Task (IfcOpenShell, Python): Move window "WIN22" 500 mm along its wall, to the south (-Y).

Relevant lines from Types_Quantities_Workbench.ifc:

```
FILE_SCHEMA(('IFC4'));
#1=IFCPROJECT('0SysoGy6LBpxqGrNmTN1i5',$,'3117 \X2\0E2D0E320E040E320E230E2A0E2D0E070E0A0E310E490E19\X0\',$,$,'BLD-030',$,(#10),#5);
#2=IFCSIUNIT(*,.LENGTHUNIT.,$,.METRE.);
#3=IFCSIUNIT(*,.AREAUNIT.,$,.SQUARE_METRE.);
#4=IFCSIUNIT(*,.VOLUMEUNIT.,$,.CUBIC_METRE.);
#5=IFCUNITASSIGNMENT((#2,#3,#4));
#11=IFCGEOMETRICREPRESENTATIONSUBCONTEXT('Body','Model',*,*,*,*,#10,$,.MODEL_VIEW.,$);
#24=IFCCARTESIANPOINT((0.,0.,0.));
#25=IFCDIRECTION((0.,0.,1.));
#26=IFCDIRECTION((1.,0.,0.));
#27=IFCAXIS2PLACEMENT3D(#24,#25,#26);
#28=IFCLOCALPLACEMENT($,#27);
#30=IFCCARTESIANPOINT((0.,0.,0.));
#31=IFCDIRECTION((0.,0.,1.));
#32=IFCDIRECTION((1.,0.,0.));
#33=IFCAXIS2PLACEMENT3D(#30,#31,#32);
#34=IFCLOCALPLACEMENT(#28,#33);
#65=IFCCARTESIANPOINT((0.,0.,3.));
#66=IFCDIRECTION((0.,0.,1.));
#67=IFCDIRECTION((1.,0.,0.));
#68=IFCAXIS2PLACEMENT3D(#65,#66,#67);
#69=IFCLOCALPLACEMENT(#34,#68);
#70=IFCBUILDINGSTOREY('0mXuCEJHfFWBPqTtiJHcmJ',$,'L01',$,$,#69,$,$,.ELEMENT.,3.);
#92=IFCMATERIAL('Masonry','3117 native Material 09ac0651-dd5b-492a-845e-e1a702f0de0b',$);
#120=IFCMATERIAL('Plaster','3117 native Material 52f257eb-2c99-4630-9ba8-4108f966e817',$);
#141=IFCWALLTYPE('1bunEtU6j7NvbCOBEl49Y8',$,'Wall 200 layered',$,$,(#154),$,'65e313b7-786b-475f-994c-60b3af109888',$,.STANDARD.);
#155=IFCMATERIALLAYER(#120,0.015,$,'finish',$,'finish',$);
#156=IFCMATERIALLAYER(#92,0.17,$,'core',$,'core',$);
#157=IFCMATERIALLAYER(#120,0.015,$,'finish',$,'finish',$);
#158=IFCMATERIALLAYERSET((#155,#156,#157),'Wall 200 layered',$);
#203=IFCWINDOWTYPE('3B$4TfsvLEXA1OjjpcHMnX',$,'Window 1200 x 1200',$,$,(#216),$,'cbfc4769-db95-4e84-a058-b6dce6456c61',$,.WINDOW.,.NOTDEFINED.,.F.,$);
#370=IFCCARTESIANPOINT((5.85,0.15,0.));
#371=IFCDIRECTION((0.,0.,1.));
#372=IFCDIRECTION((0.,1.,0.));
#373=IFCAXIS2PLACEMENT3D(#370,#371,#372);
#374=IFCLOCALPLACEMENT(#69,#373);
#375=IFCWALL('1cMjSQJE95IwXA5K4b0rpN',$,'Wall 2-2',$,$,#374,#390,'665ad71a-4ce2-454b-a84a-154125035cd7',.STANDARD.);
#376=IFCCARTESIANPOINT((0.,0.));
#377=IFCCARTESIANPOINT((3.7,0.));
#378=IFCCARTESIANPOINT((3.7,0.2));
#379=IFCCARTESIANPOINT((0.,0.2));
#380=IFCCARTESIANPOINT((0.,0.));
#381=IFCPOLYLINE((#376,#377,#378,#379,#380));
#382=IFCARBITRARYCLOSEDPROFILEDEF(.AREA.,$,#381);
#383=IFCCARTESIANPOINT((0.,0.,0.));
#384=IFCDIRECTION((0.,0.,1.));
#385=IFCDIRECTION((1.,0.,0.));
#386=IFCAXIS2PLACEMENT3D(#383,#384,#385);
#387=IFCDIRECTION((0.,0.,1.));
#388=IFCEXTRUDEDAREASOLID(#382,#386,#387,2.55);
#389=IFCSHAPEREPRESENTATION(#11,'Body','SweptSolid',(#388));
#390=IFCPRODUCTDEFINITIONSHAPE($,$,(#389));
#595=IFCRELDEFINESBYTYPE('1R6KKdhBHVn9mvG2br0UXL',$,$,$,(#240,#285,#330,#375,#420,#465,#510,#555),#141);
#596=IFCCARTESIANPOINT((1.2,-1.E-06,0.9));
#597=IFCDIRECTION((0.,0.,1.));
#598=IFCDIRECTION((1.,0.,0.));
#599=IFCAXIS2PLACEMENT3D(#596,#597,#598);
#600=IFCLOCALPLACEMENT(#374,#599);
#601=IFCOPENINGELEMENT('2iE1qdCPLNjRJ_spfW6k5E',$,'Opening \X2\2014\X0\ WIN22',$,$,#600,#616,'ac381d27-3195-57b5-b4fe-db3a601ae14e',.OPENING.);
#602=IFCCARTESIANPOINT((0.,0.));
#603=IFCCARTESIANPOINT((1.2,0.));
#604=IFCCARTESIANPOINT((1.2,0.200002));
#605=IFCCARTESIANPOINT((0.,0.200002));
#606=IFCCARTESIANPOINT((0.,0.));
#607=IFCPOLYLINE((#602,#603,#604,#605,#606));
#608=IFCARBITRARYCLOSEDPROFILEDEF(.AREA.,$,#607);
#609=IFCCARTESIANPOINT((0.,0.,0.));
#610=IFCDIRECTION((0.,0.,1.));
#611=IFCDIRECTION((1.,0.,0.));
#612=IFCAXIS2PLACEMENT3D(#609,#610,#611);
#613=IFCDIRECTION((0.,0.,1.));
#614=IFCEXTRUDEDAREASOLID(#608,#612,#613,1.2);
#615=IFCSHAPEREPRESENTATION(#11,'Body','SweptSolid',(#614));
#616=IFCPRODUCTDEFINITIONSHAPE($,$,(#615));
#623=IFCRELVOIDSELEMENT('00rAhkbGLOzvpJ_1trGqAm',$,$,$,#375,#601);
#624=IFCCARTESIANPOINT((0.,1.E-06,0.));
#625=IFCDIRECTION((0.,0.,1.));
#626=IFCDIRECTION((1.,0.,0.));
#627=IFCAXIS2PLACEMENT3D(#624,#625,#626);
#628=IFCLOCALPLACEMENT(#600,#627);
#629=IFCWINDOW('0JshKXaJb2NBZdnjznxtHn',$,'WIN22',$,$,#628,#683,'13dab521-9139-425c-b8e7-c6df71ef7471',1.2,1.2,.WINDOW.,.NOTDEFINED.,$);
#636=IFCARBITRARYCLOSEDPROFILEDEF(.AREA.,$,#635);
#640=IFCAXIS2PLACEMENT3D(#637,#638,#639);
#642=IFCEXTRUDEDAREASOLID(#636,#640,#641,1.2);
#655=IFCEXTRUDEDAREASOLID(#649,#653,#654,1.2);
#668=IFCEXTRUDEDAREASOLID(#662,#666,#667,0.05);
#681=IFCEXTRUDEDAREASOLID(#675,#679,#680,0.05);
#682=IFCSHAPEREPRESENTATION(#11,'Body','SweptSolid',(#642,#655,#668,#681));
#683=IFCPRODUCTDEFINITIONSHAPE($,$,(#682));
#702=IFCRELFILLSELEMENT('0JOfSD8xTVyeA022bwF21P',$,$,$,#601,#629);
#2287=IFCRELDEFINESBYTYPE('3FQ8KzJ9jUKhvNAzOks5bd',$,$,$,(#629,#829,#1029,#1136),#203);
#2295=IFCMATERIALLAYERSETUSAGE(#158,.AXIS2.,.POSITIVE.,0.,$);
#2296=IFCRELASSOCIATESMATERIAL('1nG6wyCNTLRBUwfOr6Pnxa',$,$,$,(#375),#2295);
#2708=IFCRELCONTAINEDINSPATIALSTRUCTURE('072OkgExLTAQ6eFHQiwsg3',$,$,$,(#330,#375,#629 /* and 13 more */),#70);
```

```python
import ifcopenshell
import ifcopenshell.api.geometry
import ifcopenshell.util.placement

model = ifcopenshell.open("Types_Quantities_Workbench.ifc")

window = model.by_id(629)
opening = window.FillsVoids[0].RelatingOpeningElement
wall = opening.VoidsElements[0].RelatingBuildingElement

wall_matrix = ifcopenshell.util.placement.get_local_placement(wall.ObjectPlacement)
shift = wall_matrix[:3, 0] * -0.5
before = ifcopenshell.util.placement.get_local_placement(window.ObjectPlacement)[:3, 3].copy()

# The window is placed relative to its opening, so it follows when the opening moves.
matrix = ifcopenshell.util.placement.get_local_placement(opening.ObjectPlacement)
matrix[:3, 3] += shift
ifcopenshell.api.geometry.edit_object_placement(
    model, product=opening, matrix=matrix, is_si=False, should_transform_children=True
)

after = ifcopenshell.util.placement.get_local_placement(window.ObjectPlacement)[:3, 3]
print("window moved by", (after - before).round(3) + 0.0)

model.write("Types_Quantities_Workbench_v2.ifc")
```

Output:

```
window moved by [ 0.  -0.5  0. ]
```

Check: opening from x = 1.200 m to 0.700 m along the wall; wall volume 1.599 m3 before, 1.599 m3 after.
